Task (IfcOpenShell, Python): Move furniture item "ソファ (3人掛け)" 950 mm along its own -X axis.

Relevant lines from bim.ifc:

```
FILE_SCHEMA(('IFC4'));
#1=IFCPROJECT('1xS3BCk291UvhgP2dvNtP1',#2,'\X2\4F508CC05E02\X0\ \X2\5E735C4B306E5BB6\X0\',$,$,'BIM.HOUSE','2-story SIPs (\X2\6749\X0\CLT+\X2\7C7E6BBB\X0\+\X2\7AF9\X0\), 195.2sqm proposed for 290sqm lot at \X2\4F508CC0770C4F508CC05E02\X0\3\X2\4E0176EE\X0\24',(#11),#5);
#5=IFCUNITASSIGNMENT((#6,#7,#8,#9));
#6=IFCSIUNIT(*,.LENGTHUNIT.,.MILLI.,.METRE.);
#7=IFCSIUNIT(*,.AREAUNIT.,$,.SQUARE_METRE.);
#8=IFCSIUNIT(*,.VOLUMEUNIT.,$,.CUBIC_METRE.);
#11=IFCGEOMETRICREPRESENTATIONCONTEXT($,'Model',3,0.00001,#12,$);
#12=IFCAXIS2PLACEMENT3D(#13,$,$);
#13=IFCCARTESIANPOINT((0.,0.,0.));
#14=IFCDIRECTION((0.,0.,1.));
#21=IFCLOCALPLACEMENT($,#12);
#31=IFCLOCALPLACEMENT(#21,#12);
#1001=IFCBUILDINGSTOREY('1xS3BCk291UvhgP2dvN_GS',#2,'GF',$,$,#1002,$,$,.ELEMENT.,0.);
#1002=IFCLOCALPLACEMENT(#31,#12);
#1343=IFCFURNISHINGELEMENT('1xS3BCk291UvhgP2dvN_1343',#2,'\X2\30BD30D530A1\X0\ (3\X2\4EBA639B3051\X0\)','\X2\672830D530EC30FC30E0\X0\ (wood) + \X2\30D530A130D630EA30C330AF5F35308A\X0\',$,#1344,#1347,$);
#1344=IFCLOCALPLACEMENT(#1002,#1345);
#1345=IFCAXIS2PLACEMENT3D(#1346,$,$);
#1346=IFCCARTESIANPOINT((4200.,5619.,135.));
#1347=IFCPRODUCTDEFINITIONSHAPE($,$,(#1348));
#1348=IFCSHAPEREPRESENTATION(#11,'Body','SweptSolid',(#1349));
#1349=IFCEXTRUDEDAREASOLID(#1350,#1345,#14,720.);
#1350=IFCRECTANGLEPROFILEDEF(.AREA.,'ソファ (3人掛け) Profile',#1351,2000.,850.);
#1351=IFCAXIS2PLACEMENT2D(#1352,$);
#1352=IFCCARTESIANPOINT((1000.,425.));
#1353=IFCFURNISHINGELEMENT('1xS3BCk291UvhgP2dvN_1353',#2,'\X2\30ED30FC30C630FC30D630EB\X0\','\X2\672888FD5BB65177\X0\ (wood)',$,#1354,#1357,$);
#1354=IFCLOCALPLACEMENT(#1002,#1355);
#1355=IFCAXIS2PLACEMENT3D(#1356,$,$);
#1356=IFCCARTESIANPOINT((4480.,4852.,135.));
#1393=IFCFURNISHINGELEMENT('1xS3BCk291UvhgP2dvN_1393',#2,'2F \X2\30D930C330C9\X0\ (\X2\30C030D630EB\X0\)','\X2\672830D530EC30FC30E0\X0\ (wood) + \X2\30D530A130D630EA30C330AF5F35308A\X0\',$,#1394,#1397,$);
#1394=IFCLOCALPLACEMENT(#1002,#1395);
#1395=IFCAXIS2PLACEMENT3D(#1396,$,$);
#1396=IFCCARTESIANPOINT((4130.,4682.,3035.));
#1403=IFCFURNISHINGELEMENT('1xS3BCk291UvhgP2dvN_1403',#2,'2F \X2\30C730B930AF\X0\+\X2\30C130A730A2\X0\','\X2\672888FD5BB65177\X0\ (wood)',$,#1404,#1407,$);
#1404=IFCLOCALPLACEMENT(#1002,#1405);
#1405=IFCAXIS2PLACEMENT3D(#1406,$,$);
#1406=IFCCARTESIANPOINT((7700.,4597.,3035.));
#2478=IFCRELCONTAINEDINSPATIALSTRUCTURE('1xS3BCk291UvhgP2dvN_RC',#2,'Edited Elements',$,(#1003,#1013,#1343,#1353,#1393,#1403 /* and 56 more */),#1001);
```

```python
import ifcopenshell
import ifcopenshell.api.geometry
import ifcopenshell.util.placement
import ifcopenshell.util.unit

model = ifcopenshell.open("bim.ifc")
unit_scale = ifcopenshell.util.unit.calculate_unit_scale(model)

item = model.by_guid("1xS3BCk291UvhgP2dvN_1343")
matrix = ifcopenshell.util.placement.get_local_placement(item.ObjectPlacement)
matrix[:3, 3] -= matrix[:3, 0] * 0.95 / unit_scale
ifcopenshell.api.geometry.edit_object_placement(model, product=item, matrix=matrix, is_si=False)

print(ifcopenshell.util.placement.get_local_placement(item.ObjectPlacement).round(3) + 0.0)

model.write("bim_rev.ifc")
```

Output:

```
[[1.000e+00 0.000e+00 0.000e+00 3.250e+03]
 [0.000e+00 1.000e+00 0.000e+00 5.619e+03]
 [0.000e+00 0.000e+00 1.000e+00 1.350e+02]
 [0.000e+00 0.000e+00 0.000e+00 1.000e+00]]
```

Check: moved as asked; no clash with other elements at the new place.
